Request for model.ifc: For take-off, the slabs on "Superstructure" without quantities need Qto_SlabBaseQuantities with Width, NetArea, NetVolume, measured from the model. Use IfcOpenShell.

First a look at what the model holds.

```python
import ifcopenshell
import ifcopenshell.util.element
import ifcopenshell.util.unit

model = ifcopenshell.open("model.ifc")
print(model.schema)
for unit_type in ("LENGTHUNIT", "AREAUNIT", "VOLUMEUNIT"):
    print(unit_type, ifcopenshell.util.unit.calculate_unit_scale(model, unit_type))
storey = next(s for s in model.by_type("IfcBuildingStorey") if s.Name == "Superstructure")
slabs = [e for e in ifcopenshell.util.element.get_decomposition(storey) if e.is_a("IfcSlab")]
for e in sorted(slabs, key=lambda e: e.id()):
    print(e.id(), e.is_a(), e.Name, list(ifcopenshell.util.element.get_psets(e, qtos_only=True)), sep=" | ")
```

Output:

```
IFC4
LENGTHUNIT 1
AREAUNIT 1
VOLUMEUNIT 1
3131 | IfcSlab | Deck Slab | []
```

```python
import ifcopenshell
import ifcopenshell.api.pset
import ifcopenshell.geom
import ifcopenshell.util.element
import ifcopenshell.util.shape
import ifcopenshell.util.unit

model = ifcopenshell.open("model.ifc")
unit_scale = ifcopenshell.util.unit.calculate_unit_scale(model)
area_scale = ifcopenshell.util.unit.calculate_unit_scale(model, "AREAUNIT")
volume_scale = ifcopenshell.util.unit.calculate_unit_scale(model, "VOLUMEUNIT")
settings = ifcopenshell.geom.settings()

storey = next(s for s in model.by_type("IfcBuildingStorey") if s.Name == "Superstructure")
slabs = [e for e in ifcopenshell.util.element.get_decomposition(storey) if e.is_a("IfcSlab")]

for e in sorted(slabs, key=lambda e: e.id()):
    if ifcopenshell.util.element.get_psets(e, qtos_only=True, should_inherit=False):
        continue
    # Geometry comes back in metres, in the element's own axes.
    shape = ifcopenshell.geom.create_shape(settings, e)
    values = {
        "Width": ifcopenshell.util.shape.get_z(shape.geometry) / unit_scale,
        "NetArea": ifcopenshell.util.shape.get_footprint_area(shape.geometry) / area_scale,
        "NetVolume": ifcopenshell.util.shape.get_volume(shape.geometry) / volume_scale,
    }
    qto = ifcopenshell.api.pset.add_qto(model, product=e, name="Qto_SlabBaseQuantities")
    ifcopenshell.api.pset.edit_qto(model, qto=qto, properties=values)
    print(e.id(), {k: round(v, 3) for k, v in values.items()})

model.write("model_rev.ifc")
```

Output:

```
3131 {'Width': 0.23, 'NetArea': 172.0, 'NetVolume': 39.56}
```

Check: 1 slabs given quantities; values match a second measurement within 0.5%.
